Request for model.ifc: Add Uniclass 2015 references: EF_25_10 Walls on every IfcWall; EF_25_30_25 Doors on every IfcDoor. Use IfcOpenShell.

First a look at what the model holds.

```python
import ifcopenshell

model = ifcopenshell.open("model.ifc")
print(model.schema)
print("classifications:", [c.Name for c in model.by_type("IfcClassification")])
for ifc_class in ("IfcDoor", "IfcRoof", "IfcStair", "IfcWall", "IfcWindow"):
    print(ifc_class, len(model.by_type(ifc_class)))
```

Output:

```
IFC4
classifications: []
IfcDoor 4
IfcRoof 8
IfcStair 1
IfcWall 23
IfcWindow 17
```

```python
import ifcopenshell
import ifcopenshell.api.classification

model = ifcopenshell.open("model.ifc")

system = ifcopenshell.api.classification.add_classification(model, classification="Uniclass 2015")

codes = {
    "IfcWall": ("EF_25_10", "Walls"),
    "IfcDoor": ("EF_25_30_25", "Doors"),
}
for ifc_class, (code, name) in codes.items():
    products = model.by_type(ifc_class)
    ifcopenshell.api.classification.add_reference(
        model, products=products, classification=system, identification=code, name=name
    )
    print(code, len(products))

model.write("model_edited.ifc")
```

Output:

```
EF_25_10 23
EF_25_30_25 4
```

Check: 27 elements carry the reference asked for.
